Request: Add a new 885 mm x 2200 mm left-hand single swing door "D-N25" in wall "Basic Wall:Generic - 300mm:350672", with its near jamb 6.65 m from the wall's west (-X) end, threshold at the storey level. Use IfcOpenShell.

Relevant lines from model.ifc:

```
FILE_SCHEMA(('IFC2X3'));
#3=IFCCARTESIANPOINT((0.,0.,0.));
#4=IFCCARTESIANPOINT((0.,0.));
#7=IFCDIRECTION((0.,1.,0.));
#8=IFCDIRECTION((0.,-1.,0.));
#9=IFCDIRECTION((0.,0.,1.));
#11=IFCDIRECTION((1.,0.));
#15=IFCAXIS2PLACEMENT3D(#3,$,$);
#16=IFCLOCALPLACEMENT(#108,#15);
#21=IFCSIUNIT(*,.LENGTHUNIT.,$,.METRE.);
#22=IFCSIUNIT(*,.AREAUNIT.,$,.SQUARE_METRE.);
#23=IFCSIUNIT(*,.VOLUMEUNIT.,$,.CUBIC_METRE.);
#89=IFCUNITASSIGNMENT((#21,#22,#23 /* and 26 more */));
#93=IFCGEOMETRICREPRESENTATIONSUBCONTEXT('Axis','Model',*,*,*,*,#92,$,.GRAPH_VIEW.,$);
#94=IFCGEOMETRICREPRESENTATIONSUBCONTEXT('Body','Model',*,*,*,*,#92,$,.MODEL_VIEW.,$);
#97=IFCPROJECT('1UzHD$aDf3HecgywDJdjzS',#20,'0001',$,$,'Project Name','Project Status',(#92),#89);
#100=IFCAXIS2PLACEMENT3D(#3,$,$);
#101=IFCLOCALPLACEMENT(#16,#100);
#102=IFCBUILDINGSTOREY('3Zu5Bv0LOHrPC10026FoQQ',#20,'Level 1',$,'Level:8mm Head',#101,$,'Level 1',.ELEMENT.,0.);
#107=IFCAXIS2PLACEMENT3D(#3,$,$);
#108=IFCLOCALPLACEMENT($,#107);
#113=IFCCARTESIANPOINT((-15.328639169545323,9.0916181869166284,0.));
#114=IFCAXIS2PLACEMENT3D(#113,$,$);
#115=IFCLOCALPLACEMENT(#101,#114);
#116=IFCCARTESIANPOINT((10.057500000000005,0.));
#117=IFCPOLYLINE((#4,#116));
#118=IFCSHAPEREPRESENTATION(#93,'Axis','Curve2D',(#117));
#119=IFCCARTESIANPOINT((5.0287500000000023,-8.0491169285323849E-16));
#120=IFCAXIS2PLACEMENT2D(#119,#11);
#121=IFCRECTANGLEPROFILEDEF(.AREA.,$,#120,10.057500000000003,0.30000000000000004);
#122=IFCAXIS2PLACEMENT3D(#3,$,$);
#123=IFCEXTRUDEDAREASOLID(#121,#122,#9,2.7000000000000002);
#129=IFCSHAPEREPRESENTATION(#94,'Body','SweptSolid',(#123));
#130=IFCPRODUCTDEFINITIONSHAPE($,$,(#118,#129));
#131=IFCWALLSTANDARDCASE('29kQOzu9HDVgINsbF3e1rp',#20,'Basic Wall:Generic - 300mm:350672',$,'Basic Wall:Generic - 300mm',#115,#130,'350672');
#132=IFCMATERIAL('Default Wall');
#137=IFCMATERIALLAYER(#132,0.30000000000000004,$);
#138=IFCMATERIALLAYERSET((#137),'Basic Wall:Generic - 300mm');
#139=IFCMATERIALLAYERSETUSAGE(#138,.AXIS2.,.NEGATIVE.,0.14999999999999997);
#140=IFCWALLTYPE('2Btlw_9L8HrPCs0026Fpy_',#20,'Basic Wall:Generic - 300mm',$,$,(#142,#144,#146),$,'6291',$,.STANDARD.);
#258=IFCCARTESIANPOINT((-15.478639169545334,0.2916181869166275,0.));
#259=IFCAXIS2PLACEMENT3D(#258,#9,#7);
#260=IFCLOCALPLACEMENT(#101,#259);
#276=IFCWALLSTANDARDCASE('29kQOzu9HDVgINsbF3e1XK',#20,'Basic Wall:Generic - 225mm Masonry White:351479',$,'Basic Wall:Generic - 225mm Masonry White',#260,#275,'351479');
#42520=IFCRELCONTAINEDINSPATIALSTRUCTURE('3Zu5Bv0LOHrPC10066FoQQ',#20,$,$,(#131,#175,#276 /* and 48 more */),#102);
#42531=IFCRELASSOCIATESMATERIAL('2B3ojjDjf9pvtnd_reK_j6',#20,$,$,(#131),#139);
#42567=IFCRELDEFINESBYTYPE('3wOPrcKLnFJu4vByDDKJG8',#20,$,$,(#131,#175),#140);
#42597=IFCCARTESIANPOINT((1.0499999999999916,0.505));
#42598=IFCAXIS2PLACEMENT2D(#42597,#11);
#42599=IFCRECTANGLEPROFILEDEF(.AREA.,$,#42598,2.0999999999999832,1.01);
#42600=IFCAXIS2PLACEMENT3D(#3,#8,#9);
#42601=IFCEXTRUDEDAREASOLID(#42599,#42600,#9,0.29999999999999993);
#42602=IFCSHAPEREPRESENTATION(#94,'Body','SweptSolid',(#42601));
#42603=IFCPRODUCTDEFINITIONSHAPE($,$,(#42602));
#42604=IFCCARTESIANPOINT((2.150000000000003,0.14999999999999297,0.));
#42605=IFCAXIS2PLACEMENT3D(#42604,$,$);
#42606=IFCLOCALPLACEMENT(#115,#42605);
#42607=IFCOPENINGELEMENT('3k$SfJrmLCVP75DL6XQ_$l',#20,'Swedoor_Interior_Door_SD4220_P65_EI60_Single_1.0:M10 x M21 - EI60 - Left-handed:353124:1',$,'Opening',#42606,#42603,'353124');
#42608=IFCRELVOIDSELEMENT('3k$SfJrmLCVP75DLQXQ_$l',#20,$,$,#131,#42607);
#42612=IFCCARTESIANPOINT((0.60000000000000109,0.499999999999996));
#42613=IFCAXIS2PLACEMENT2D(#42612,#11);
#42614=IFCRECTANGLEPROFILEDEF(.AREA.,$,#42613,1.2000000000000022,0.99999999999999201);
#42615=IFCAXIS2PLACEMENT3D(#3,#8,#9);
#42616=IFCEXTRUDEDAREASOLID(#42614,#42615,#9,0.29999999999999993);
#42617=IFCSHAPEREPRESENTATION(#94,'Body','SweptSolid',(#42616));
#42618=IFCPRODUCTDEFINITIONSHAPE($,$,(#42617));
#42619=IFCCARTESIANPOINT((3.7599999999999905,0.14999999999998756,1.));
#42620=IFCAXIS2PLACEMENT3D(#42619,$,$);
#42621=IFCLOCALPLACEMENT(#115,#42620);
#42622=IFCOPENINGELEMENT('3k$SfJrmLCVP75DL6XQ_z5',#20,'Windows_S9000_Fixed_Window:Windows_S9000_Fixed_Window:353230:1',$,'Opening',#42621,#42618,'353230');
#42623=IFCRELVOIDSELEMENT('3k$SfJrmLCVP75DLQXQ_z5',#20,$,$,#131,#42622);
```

```python
import numpy as np
import ifcopenshell
import ifcopenshell.api.feature
import ifcopenshell.api.geometry
import ifcopenshell.api.root
import ifcopenshell.api.spatial
import ifcopenshell.api.type
import ifcopenshell.geom
import ifcopenshell.util.element
import ifcopenshell.util.placement
import ifcopenshell.util.representation
import ifcopenshell.util.shape
import ifcopenshell.util.unit

model = ifcopenshell.open("model.ifc")
unit_scale = ifcopenshell.util.unit.calculate_unit_scale(model)
settings = ifcopenshell.geom.settings()


def volume(element):
    """Net volume in cubic metres, openings subtracted."""
    shape = ifcopenshell.geom.create_shape(settings, element)
    return ifcopenshell.util.shape.get_volume(shape.geometry)


wall = model.by_guid("29kQOzu9HDVgINsbF3e1rp")
storey = ifcopenshell.util.element.get_container(wall, ifc_class="IfcBuildingStorey")
context = ifcopenshell.util.representation.get_context(model, "Model", "Body", "MODEL_VIEW")
before = volume(wall)

width, height, from_end, sill = 0.885, 2.2, 6.65, 0.0  # metres

# The wall runs along its own X axis, and the end named is its -X end.
wall_shape = ifcopenshell.geom.create_shape(settings, wall)
x, y, z = ifcopenshell.util.shape.get_vertices(wall_shape.geometry).T
start = x.min() + from_end
face, thickness = float(y.min()), float(y.max() - y.min())
wall_matrix = ifcopenshell.util.placement.get_local_placement(wall.ObjectPlacement)
level = ifcopenshell.util.placement.get_local_placement(storey.ObjectPlacement)[2, 3]


def in_wall(x, y):
    """Placement at x, y metres in the wall's axes, at sill height."""
    matrix = wall_matrix.copy()
    matrix[:, 3] = wall_matrix @ np.array([x / unit_scale, y / unit_scale, 0.0, 1.0])
    matrix[2, 3] = level + sill / unit_scale
    return matrix


# Opening: a box that overshoots both wall faces by 50 mm.
opening = ifcopenshell.api.root.create_entity(model, ifc_class="IfcOpeningElement")
box = ifcopenshell.api.geometry.add_wall_representation(
    model, context=context, length=width, height=height, thickness=thickness + 0.1
)
ifcopenshell.api.geometry.assign_representation(model, product=opening, representation=box)
ifcopenshell.api.geometry.edit_object_placement(model, product=opening, matrix=in_wall(start, face - 0.05), is_si=False)
ifcopenshell.api.feature.add_feature(model, feature=opening, element=wall)

door = ifcopenshell.api.root.create_entity(model, ifc_class="IfcDoor", name="D-N25")
door.OverallWidth, door.OverallHeight = width / unit_scale, height / unit_scale
body = ifcopenshell.api.geometry.add_door_representation(
    model,
    context=context,
    overall_width=door.OverallWidth,
    overall_height=door.OverallHeight,
    operation_type="SINGLE_SWING_LEFT",
    lining_properties={"LiningDepth": thickness / unit_scale, "ThresholdDepth": thickness / unit_scale},
)
ifcopenshell.api.geometry.assign_representation(model, product=door, representation=body)
ifcopenshell.api.spatial.assign_container(model, products=[door], relating_structure=storey)
fills = ifcopenshell.api.feature.add_filling(model, opening=opening, element=door)
fills.OwnerHistory = door.OwnerHistory  # required in IFC2X3

# IFC2X3 keeps the operation on the door style.
style = ifcopenshell.api.root.create_entity(model, ifc_class="IfcDoorStyle", name="D-N25")
style.OperationType, style.ConstructionType = "SINGLE_SWING_LEFT", "NOTDEFINED"
style.ParameterTakesPrecedence = style.Sizeable = False
ifcopenshell.api.type.assign_type(model, related_objects=[door], relating_type=style)

# The lining spans the wall, so the door starts at the wall face.
ifcopenshell.api.geometry.edit_object_placement(model, product=door, matrix=in_wall(start, face), is_si=False)

after = volume(wall)

print(f"wall volume {before:.3f} -> {after:.3f} m3")

model.write("model_edited.ifc")
```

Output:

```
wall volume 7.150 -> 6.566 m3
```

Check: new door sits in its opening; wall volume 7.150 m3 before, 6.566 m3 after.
